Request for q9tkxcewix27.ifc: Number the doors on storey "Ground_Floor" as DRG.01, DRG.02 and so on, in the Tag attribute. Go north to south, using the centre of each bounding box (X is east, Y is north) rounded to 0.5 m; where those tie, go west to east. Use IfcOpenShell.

First a look at what the model holds.

```python
import ifcopenshell
import ifcopenshell.util.element
import ifcopenshell.util.placement

model = ifcopenshell.open("q9tkxcewix27.ifc")
print(model.schema)
storey = next(s for s in model.by_type("IfcBuildingStorey") if s.Name == "Ground_Floor")
doors = [e for e in ifcopenshell.util.element.get_decomposition(storey) if e.is_a("IfcDoor")]
for e in sorted(doors, key=lambda e: e.id()):
    origin = ifcopenshell.util.placement.get_local_placement(e.ObjectPlacement)[:3, 3]
    print(e.id(), e.Tag, e.Name, origin.round(2) + 0.0, sep=" | ")
```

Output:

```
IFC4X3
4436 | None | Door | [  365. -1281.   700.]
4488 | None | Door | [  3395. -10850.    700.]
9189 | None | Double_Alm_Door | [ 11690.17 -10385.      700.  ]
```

```python
import ifcopenshell
import ifcopenshell.geom
import ifcopenshell.util.element
import ifcopenshell.util.shape

model = ifcopenshell.open("q9tkxcewix27.ifc")
settings = ifcopenshell.geom.settings()
settings.set("use-world-coords", True)


def centre(element):
    shape = ifcopenshell.geom.create_shape(settings, element)
    return ifcopenshell.util.shape.get_bbox_centroid(shape.geometry)


storey = next(s for s in model.by_type("IfcBuildingStorey") if s.Name == "Ground_Floor")
doors = [e for e in ifcopenshell.util.element.get_decomposition(storey) if e.is_a("IfcDoor")]

# Insertion points can sit at a corner or the storey origin, so sort by the geometry (in metres).
centres = {e: centre(e) for e in doors}
doors.sort(key=lambda e: (-round(centres[e][1] / 0.5), centres[e][0]))

for i, e in enumerate(doors, start=1):
    number = f"DRG.{i:02d}"
    e.Tag = number
    print(e.id(), number)

model.write("q9tkxcewix27_updated.ifc")
```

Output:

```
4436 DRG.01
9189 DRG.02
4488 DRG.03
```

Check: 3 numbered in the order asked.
